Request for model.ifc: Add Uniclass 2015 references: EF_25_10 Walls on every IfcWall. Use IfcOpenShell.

First a look at what the model holds.

```python
import ifcopenshell

model = ifcopenshell.open("model.ifc")
print(model.schema)
print("classifications:", [c.Name for c in model.by_type("IfcClassification")])
for ifc_class in ("IfcDoor", "IfcRoof", "IfcStair", "IfcWall", "IfcWindow"):
    print(ifc_class, len(model.by_type(ifc_class)))
```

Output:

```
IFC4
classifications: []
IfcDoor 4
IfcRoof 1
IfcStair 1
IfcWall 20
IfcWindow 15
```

```python
import ifcopenshell
import ifcopenshell.api.classification

model = ifcopenshell.open("model.ifc")

system = ifcopenshell.api.classification.add_classification(model, classification="Uniclass 2015")

codes = {
    "IfcWall": ("EF_25_10", "Walls"),
}
for ifc_class, (code, name) in codes.items():
    products = model.by_type(ifc_class)
    ifcopenshell.api.classification.add_reference(
        model, products=products, classification=system, identification=code, name=name
    )
    print(code, len(products))

model.write("model-out.ifc")
```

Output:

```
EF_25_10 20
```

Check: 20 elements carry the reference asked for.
